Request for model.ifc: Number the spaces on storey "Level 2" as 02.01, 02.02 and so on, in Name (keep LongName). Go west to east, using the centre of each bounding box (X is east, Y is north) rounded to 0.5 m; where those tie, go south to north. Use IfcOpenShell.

First a look at what the model holds.

```python
import ifcopenshell
import ifcopenshell.util.element
import ifcopenshell.util.placement

model = ifcopenshell.open("model.ifc")
print(model.schema)
storey = next(s for s in model.by_type("IfcBuildingStorey") if s.Name == "Level 2")
spaces = [e for e in ifcopenshell.util.element.get_decomposition(storey) if e.is_a("IfcSpace")]
for e in sorted(spaces, key=lambda e: e.id()):
    origin = ifcopenshell.util.placement.get_local_placement(e.ObjectPlacement)[:3, 3]
    print(e.id(), e.Name, e.LongName, origin.round(2) + 0.0, sep=" | ")
```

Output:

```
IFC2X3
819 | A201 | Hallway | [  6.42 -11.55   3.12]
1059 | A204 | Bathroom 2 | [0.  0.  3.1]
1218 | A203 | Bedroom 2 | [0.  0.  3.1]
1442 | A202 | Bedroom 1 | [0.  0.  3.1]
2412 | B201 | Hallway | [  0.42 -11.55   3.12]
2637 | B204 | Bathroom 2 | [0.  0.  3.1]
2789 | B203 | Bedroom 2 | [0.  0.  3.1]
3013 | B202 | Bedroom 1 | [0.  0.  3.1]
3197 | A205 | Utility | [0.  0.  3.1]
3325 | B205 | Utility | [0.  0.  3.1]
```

```python
import ifcopenshell
import ifcopenshell.geom
import ifcopenshell.util.element
import ifcopenshell.util.shape

model = ifcopenshell.open("model.ifc")
settings = ifcopenshell.geom.settings()
settings.set("use-world-coords", True)


def centre(element):
    shape = ifcopenshell.geom.create_shape(settings, element)
    return ifcopenshell.util.shape.get_bbox_centroid(shape.geometry)


storey = next(s for s in model.by_type("IfcBuildingStorey") if s.Name == "Level 2")
spaces = [e for e in ifcopenshell.util.element.get_decomposition(storey) if e.is_a("IfcSpace")]

# Insertion points can sit at a corner or the storey origin, so sort by the geometry (in metres).
centres = {e: centre(e) for e in spaces}
spaces.sort(key=lambda e: (round(centres[e][0] / 0.5), centres[e][1]))

for i, e in enumerate(spaces, start=1):
    number = f"02.{i:02d}"
    e.Name = number
    print(e.id(), number)

model.write("model_rev.ifc")
```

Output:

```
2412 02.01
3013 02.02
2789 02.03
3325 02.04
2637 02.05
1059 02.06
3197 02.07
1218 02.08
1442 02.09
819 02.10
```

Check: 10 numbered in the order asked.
